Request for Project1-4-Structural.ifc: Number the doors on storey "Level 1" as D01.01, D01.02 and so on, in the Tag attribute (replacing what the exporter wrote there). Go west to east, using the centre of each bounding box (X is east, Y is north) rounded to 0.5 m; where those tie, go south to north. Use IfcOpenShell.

First a look at what the model holds.

```python
import ifcopenshell
import ifcopenshell.util.element
import ifcopenshell.util.placement

model = ifcopenshell.open("Project1-4-Structural.ifc")
print(model.schema)
storey = next(s for s in model.by_type("IfcBuildingStorey") if s.Name == "Level 1")
doors = [e for e in ifcopenshell.util.element.get_decomposition(storey) if e.is_a("IfcDoor")]
for e in sorted(doors, key=lambda e: e.id()):
    origin = ifcopenshell.util.placement.get_local_placement(e.ObjectPlacement)[:3, 3]
    print(e.id(), e.Tag, e.Name, origin.round(2) + 0.0, sep=" | ")
```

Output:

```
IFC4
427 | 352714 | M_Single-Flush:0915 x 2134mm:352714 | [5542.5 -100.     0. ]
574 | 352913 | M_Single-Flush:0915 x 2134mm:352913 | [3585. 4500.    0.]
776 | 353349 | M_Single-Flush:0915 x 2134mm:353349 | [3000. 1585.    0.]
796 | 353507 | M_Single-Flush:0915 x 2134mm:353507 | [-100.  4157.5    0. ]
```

```python
import ifcopenshell
import ifcopenshell.geom
import ifcopenshell.util.element
import ifcopenshell.util.shape

model = ifcopenshell.open("Project1-4-Structural.ifc")
settings = ifcopenshell.geom.settings()
settings.set("use-world-coords", True)


def centre(element):
    shape = ifcopenshell.geom.create_shape(settings, element)
    return ifcopenshell.util.shape.get_bbox_centroid(shape.geometry)


storey = next(s for s in model.by_type("IfcBuildingStorey") if s.Name == "Level 1")
doors = [e for e in ifcopenshell.util.element.get_decomposition(storey) if e.is_a("IfcDoor")]

# Insertion points can sit at a corner or the storey origin, so sort by the geometry (in metres).
centres = {e: centre(e) for e in doors}
doors.sort(key=lambda e: (round(centres[e][0] / 0.5), centres[e][1]))

for i, e in enumerate(doors, start=1):
    number = f"D01.{i:02d}"
    e.Tag = number
    print(e.id(), number)

model.write("Project1-4-Structural_rev.ifc")
```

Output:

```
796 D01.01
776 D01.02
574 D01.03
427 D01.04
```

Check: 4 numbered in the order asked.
